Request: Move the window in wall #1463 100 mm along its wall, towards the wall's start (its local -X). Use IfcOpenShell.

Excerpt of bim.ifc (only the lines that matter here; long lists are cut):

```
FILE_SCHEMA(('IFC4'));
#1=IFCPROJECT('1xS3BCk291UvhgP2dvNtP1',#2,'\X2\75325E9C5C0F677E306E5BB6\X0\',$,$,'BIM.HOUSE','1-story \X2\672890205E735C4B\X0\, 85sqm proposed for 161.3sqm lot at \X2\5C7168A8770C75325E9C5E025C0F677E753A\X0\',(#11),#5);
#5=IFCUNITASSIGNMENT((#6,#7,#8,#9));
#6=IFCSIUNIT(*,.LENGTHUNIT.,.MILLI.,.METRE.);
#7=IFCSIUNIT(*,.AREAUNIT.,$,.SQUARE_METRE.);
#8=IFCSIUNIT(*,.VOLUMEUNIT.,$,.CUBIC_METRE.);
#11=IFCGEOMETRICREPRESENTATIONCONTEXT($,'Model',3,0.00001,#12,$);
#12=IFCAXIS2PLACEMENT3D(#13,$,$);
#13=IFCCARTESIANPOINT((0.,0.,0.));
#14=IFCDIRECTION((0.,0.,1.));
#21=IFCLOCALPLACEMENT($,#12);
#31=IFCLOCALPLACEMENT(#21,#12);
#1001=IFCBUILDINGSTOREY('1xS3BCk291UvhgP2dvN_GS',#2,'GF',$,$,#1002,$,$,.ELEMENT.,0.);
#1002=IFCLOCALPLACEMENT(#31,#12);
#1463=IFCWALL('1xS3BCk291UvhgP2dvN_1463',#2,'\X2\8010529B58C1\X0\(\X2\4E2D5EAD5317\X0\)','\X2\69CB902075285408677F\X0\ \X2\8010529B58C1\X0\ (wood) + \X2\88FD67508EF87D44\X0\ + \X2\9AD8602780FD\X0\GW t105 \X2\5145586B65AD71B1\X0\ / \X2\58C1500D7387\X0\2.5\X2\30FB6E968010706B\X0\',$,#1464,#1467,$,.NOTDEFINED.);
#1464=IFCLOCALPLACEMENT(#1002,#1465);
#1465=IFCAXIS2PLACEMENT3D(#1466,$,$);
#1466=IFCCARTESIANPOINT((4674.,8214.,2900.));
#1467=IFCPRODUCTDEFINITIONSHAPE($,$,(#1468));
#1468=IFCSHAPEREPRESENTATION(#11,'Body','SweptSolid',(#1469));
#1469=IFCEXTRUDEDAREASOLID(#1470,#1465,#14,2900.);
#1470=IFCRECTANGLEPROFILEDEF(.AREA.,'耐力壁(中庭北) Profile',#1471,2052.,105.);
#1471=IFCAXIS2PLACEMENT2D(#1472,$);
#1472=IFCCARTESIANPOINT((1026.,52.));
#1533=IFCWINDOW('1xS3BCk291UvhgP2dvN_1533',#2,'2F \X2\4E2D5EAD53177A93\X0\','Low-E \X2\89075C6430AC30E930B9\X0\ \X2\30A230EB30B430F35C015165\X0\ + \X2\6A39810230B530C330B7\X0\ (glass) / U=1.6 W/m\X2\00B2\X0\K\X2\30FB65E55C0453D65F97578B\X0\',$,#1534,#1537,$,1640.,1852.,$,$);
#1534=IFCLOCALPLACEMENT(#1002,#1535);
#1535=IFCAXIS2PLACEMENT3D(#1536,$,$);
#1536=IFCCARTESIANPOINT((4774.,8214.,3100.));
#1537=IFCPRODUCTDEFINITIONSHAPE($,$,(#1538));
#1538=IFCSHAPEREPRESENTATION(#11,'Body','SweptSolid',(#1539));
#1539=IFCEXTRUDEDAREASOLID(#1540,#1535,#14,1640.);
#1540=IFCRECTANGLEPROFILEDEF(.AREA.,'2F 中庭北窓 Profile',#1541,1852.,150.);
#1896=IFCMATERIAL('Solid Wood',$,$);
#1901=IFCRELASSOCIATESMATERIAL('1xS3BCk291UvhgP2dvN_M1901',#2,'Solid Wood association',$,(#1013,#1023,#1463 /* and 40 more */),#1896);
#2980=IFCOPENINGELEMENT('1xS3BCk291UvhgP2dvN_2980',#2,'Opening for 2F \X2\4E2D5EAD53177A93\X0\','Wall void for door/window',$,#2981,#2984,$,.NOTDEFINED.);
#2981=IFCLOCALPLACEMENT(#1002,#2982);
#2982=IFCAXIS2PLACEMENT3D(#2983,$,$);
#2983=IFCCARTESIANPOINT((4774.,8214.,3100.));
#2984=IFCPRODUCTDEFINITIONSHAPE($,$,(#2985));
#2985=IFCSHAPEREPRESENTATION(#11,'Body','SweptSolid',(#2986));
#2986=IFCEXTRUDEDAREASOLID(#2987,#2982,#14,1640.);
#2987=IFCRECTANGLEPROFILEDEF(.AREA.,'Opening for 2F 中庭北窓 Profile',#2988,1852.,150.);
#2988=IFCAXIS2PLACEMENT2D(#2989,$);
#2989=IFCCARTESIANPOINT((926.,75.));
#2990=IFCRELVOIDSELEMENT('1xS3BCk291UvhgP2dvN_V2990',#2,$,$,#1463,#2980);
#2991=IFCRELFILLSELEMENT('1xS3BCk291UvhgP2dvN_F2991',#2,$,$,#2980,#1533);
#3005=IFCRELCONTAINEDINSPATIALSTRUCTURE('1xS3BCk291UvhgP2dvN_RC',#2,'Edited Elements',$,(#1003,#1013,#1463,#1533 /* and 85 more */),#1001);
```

```python
import ifcopenshell
import ifcopenshell.api.geometry
import ifcopenshell.util.placement

model = ifcopenshell.open("bim.ifc")

window = model.by_guid("1xS3BCk291UvhgP2dvN_1533")
opening = window.FillsVoids[0].RelatingOpeningElement
wall = opening.VoidsElements[0].RelatingBuildingElement

wall_matrix = ifcopenshell.util.placement.get_local_placement(wall.ObjectPlacement)
shift = wall_matrix[:3, 0] * -100.0
before = ifcopenshell.util.placement.get_local_placement(window.ObjectPlacement)[:3, 3].copy()

# The window is not placed relative to its opening, so move both.
for product in (opening, window):
    matrix = ifcopenshell.util.placement.get_local_placement(product.ObjectPlacement)
    matrix[:3, 3] += shift
    ifcopenshell.api.geometry.edit_object_placement(model, product=product, matrix=matrix, is_si=False)

after = ifcopenshell.util.placement.get_local_placement(window.ObjectPlacement)[:3, 3]
print("window moved by", (after - before).round(3) + 0.0)

model.write("bim-out.ifc")
```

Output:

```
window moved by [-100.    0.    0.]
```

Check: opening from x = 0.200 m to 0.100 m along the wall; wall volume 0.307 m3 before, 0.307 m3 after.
